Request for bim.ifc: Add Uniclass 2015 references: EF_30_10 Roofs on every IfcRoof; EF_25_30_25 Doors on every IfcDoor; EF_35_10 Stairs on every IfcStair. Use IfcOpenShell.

First a look at what the model holds.

```python
import ifcopenshell

model = ifcopenshell.open("bim.ifc")
print(model.schema)
print("classifications:", [c.Name for c in model.by_type("IfcClassification")])
for ifc_class in ("IfcDoor", "IfcRoof", "IfcStair", "IfcWall", "IfcWindow"):
    print(ifc_class, len(model.by_type(ifc_class)))
```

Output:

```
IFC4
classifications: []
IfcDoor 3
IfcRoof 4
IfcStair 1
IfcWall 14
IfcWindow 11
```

```python
import ifcopenshell
import ifcopenshell.api.classification

model = ifcopenshell.open("bim.ifc")

system = ifcopenshell.api.classification.add_classification(model, classification="Uniclass 2015")

codes = {
    "IfcRoof": ("EF_30_10", "Roofs"),
    "IfcDoor": ("EF_25_30_25", "Doors"),
    "IfcStair": ("EF_35_10", "Stairs"),
}
for ifc_class, (code, name) in codes.items():
    products = model.by_type(ifc_class)
    ifcopenshell.api.classification.add_reference(
        model, products=products, classification=system, identification=code, name=name
    )
    print(code, len(products))

model.write("bim_v2.ifc")
```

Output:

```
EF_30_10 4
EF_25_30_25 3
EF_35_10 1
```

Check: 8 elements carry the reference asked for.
